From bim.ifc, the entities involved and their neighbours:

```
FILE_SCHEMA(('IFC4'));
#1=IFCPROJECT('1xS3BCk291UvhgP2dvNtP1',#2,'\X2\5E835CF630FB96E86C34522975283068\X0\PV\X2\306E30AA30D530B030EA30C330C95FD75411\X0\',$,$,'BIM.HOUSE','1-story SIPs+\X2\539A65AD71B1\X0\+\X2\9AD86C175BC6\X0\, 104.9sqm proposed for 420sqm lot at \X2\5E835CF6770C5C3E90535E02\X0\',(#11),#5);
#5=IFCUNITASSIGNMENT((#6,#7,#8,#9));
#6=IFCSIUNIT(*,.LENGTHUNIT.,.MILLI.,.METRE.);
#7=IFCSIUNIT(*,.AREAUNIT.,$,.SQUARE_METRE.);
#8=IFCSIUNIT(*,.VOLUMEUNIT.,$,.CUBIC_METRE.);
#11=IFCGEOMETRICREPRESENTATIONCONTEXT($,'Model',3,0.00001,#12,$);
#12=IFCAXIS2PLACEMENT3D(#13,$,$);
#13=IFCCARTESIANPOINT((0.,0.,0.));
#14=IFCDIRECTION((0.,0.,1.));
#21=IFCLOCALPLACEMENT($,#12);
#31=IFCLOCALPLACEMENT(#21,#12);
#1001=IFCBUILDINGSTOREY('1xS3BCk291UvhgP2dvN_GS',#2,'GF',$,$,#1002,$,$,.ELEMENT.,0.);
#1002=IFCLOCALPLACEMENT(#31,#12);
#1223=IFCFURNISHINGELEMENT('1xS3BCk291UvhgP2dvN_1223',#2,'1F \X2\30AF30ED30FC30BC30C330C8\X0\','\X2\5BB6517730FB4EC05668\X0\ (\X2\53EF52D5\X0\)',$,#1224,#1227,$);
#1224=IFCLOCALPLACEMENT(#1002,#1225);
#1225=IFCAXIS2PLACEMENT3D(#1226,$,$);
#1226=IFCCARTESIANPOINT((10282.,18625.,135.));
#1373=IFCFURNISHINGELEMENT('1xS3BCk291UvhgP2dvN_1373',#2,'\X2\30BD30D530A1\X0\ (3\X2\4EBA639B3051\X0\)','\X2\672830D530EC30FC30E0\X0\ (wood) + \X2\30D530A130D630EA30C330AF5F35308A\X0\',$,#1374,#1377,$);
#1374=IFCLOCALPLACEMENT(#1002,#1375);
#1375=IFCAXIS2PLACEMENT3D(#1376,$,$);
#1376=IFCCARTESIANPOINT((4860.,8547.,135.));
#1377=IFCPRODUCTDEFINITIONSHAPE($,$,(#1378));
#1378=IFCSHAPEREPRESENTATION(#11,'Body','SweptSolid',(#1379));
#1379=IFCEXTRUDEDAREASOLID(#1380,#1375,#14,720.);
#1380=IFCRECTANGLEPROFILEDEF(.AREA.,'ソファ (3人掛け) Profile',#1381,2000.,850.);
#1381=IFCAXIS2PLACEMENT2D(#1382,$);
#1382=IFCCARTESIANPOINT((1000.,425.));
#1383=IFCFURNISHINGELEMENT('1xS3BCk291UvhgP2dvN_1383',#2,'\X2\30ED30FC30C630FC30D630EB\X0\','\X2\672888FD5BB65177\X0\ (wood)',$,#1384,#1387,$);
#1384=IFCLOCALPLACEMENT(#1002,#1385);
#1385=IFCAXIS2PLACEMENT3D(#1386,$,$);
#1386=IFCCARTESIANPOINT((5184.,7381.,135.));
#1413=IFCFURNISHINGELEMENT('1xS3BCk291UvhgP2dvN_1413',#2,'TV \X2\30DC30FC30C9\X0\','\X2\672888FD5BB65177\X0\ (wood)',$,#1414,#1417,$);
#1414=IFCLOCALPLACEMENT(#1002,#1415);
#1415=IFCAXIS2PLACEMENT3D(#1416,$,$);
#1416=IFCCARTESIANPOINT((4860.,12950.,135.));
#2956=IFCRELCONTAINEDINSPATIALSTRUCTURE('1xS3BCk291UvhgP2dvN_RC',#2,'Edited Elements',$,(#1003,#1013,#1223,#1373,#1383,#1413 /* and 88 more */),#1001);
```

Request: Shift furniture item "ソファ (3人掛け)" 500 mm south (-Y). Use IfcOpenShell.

```python
import ifcopenshell
import ifcopenshell.api.geometry
import ifcopenshell.util.placement

model = ifcopenshell.open("bim.ifc")

item = model.by_id(1373)
matrix = ifcopenshell.util.placement.get_local_placement(item.ObjectPlacement)
matrix[1, 3] -= 500.0
ifcopenshell.api.geometry.edit_object_placement(model, product=item, matrix=matrix, is_si=False)

print(ifcopenshell.util.placement.get_local_placement(item.ObjectPlacement).round(3) + 0.0)

model.write("bim_v2.ifc")
```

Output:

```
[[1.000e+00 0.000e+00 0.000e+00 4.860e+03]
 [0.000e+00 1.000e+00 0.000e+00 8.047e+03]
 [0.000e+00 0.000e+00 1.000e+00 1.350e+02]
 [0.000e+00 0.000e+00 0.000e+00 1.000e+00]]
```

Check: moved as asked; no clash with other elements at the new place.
